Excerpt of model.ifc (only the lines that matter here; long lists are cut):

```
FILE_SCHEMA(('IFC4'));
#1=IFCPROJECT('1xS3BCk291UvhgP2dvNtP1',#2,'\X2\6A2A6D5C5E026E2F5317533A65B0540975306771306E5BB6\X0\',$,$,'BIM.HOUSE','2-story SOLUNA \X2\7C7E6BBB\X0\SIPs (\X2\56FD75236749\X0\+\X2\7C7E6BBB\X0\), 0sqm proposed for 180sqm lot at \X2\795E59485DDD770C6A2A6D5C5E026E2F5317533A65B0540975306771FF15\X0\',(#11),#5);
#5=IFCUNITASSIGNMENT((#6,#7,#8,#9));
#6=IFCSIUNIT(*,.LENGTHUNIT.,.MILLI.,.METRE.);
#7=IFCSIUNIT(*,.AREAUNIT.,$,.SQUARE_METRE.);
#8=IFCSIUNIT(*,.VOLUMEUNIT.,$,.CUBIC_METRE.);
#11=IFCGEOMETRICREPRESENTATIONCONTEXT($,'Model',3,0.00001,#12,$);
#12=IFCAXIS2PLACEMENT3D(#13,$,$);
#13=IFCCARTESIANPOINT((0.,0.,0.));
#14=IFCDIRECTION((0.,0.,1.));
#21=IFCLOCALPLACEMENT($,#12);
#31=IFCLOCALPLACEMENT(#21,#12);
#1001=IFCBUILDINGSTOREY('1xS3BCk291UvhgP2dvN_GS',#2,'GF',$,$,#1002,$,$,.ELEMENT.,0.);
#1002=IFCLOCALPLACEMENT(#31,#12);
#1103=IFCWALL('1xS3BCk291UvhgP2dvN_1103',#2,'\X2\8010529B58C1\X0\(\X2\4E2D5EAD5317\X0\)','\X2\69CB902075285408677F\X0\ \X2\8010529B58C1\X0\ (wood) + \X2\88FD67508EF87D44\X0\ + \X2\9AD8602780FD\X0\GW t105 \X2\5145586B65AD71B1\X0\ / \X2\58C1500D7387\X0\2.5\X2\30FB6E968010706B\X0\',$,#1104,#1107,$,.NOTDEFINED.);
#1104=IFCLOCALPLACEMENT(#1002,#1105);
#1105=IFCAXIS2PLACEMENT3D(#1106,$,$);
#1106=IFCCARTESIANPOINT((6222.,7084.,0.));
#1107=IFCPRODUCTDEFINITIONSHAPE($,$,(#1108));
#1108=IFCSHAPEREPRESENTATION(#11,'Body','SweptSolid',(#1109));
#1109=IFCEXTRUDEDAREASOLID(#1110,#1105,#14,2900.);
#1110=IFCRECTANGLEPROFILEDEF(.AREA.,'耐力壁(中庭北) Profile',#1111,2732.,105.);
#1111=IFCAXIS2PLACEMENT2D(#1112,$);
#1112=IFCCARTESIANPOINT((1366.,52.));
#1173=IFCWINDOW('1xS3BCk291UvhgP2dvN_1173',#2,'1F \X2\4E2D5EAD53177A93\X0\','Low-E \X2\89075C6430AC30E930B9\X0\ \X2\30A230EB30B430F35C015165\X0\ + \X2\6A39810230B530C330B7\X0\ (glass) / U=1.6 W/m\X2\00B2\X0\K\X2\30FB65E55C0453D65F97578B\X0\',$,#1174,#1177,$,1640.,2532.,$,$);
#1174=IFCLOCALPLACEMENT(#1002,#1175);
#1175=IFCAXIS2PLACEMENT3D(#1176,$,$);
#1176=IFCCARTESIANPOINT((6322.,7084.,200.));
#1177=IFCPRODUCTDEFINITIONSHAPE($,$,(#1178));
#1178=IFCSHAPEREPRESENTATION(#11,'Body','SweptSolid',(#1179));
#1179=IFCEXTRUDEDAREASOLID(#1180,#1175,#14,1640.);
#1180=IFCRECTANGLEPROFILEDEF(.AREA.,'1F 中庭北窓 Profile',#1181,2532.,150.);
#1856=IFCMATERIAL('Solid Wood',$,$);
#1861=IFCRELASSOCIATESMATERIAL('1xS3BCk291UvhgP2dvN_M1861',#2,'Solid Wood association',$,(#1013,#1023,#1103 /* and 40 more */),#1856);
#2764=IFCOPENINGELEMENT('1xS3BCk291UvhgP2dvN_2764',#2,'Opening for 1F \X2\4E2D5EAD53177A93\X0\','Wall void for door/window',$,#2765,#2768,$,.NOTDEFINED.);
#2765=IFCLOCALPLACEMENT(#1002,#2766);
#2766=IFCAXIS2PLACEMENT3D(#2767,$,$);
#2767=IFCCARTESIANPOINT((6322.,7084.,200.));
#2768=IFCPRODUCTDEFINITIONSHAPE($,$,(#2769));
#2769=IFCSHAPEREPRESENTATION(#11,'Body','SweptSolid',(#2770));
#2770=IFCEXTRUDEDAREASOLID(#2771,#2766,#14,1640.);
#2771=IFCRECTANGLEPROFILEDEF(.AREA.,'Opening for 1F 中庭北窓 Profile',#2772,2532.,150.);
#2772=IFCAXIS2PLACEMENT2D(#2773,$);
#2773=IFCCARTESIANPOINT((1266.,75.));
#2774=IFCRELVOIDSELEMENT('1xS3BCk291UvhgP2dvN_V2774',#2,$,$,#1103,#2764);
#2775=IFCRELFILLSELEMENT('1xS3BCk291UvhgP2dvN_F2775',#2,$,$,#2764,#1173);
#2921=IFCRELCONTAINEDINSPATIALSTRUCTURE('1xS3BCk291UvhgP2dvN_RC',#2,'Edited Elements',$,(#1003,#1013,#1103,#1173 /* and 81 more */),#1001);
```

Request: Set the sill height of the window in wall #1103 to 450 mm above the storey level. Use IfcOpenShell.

```python
import numpy as np
import ifcopenshell
import ifcopenshell.api.geometry
import ifcopenshell.geom
import ifcopenshell.util.element
import ifcopenshell.util.placement
import ifcopenshell.util.shape
import ifcopenshell.util.unit

model = ifcopenshell.open("model.ifc")
unit_scale = ifcopenshell.util.unit.calculate_unit_scale(model)

window = model.by_guid("1xS3BCk291UvhgP2dvN_1173")
opening = window.FillsVoids[0].RelatingOpeningElement
storey = ifcopenshell.util.element.get_container(window, ifc_class="IfcBuildingStorey")
level = ifcopenshell.util.placement.get_local_placement(storey.ObjectPlacement)[2, 3]

# The opening's origin need not be at the sill, so measure its lowest point.
shape = ifcopenshell.geom.create_shape(ifcopenshell.geom.settings(), opening)
bottom = ifcopenshell.util.shape.get_shape_bottom_elevation(shape, shape.geometry) / unit_scale
dz = level + 450.0 - bottom

shift = np.array([0.0, 0.0, dz])
# The window is not placed relative to its opening, so move both.
for product in (opening, window):
    matrix = ifcopenshell.util.placement.get_local_placement(product.ObjectPlacement)
    matrix[:3, 3] += shift
    ifcopenshell.api.geometry.edit_object_placement(model, product=product, matrix=matrix, is_si=False)

print(f"moved by {dz * unit_scale:+.3f} m")

model.write("model_updated.ifc")
```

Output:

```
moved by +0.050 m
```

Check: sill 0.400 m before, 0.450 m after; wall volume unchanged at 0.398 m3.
